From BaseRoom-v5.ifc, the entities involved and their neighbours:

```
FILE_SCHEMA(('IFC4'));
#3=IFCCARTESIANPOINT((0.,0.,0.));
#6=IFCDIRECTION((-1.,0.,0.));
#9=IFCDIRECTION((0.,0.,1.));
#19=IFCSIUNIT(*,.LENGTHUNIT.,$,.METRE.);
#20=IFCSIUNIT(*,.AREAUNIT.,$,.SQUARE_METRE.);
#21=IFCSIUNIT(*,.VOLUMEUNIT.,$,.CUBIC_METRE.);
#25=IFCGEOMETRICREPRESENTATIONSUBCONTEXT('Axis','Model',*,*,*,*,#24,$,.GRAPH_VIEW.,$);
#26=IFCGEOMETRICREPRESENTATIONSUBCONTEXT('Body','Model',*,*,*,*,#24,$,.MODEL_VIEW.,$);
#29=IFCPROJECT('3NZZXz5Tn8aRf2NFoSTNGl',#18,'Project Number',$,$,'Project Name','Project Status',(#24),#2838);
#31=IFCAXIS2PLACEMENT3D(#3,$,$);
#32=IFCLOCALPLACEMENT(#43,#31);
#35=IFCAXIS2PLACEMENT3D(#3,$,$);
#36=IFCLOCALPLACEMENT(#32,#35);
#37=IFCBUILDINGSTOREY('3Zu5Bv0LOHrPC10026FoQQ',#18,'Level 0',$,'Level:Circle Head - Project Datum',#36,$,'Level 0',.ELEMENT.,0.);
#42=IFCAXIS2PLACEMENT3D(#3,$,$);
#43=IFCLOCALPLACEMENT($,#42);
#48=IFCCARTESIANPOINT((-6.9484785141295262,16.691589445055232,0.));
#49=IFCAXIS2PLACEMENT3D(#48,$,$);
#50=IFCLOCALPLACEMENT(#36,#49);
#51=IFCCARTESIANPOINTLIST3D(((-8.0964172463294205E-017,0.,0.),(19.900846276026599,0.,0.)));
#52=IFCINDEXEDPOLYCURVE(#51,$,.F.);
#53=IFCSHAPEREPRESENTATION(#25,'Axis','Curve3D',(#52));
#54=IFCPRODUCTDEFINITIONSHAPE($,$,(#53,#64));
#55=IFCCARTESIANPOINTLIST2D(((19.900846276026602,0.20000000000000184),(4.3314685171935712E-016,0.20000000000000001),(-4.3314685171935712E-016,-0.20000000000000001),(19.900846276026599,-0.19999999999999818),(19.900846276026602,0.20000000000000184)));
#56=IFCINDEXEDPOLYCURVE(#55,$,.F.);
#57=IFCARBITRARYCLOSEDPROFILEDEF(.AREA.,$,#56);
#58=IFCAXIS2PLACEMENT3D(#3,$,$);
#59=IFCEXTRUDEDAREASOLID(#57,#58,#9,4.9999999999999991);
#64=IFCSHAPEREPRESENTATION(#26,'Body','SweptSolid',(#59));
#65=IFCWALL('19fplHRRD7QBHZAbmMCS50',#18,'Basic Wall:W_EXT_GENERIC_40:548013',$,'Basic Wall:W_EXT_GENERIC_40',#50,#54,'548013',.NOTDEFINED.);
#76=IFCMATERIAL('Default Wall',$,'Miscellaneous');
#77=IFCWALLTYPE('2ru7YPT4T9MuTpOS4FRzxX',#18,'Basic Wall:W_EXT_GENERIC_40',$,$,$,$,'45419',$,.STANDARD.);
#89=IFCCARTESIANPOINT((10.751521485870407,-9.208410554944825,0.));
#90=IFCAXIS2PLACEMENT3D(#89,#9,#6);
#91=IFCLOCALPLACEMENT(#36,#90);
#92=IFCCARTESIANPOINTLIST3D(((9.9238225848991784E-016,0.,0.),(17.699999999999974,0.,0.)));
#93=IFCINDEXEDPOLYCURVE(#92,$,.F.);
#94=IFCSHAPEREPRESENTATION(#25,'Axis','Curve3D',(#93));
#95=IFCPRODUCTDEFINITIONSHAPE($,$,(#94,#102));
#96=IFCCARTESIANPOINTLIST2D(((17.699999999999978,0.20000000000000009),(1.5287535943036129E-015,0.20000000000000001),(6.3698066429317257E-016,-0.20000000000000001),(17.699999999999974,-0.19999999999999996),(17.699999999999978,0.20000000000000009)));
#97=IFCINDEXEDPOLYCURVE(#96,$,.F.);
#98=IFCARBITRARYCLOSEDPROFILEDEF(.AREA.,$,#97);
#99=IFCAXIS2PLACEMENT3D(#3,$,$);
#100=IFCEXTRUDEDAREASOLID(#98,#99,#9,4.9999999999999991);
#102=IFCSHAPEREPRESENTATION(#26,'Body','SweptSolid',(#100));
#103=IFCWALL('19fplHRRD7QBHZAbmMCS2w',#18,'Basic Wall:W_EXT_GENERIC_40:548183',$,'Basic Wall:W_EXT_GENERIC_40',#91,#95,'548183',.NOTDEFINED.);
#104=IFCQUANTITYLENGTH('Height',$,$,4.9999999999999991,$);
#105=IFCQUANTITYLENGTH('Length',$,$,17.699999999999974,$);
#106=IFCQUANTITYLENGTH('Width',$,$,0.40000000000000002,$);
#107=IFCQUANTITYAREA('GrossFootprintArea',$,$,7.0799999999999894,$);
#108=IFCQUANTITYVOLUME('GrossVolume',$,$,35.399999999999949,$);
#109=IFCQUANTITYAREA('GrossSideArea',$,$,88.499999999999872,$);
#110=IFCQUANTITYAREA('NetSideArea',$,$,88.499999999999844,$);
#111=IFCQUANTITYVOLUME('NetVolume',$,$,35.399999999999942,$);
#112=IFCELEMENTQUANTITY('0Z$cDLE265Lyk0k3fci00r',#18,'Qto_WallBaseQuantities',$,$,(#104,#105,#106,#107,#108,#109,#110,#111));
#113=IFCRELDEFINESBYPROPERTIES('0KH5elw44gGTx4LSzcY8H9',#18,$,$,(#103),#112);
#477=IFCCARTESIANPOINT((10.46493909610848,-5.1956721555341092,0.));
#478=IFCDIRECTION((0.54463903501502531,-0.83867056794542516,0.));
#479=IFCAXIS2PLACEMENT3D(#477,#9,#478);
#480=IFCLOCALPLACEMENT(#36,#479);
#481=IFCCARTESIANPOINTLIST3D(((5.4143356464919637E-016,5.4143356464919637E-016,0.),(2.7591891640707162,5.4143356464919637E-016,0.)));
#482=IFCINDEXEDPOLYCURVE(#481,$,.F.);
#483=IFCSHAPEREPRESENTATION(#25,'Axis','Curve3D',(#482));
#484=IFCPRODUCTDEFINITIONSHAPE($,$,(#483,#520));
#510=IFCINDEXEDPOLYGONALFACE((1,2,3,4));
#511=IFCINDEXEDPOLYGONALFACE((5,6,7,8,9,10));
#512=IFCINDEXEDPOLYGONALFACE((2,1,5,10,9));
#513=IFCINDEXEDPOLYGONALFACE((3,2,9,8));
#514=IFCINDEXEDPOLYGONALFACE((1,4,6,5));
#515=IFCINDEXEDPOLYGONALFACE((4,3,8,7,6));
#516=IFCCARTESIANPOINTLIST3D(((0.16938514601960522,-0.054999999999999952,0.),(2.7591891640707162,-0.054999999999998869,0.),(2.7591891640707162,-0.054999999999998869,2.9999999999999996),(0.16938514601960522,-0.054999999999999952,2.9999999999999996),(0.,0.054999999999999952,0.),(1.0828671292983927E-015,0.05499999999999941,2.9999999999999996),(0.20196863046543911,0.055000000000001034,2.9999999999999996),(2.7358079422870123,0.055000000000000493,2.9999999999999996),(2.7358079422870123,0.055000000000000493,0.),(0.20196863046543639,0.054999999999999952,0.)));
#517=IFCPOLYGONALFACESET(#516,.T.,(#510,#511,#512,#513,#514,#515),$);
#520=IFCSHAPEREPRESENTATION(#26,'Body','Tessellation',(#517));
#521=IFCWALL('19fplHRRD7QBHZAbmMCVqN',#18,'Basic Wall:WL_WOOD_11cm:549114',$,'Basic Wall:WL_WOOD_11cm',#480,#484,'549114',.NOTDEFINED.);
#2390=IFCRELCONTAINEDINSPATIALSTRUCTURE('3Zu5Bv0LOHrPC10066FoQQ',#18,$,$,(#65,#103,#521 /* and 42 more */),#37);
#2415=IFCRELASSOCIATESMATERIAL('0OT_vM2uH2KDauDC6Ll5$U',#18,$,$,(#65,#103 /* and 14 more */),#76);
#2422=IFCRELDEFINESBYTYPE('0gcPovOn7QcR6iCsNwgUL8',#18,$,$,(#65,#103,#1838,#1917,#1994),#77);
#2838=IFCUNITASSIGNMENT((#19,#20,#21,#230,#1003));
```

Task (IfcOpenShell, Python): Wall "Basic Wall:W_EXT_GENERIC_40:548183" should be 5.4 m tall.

```python
import ifcopenshell
import ifcopenshell.api.pset
import ifcopenshell.geom
import ifcopenshell.util.element
import ifcopenshell.util.representation
import ifcopenshell.util.shape
import ifcopenshell.util.unit

model = ifcopenshell.open("BaseRoom-v5.ifc")
unit_scale = ifcopenshell.util.unit.calculate_unit_scale(model)
area_scale = ifcopenshell.util.unit.calculate_unit_scale(model, "AREAUNIT")
volume_scale = ifcopenshell.util.unit.calculate_unit_scale(model, "VOLUMEUNIT")
settings = ifcopenshell.geom.settings()


def volume(element):
    """Net volume in cubic metres, openings subtracted."""
    shape = ifcopenshell.geom.create_shape(settings, element)
    return ifcopenshell.util.shape.get_volume(shape.geometry)


wall = model.by_guid("19fplHRRD7QBHZAbmMCS2w")
before = volume(wall)

body = ifcopenshell.util.representation.get_representation(wall, "Model", "Body")
solid = body.Items[0]
old_height = solid.Depth
solid.Depth = 5.4
after = volume(wall)
thickness = 0.4  # wall thickness in metres

# Update the stored height, areas and volumes.
qto = model.by_id(ifcopenshell.util.element.get_pset(wall, "Qto_WallBaseQuantities", should_inherit=False)["id"])
ifcopenshell.api.pset.edit_qto(model, qto=qto, properties={
    "Height": solid.Depth,
    "GrossVolume": ifcopenshell.util.element.get_pset(wall, "Qto_WallBaseQuantities", "GrossVolume") * solid.Depth / old_height,
    "GrossSideArea": ifcopenshell.util.element.get_pset(wall, "Qto_WallBaseQuantities", "GrossSideArea") * solid.Depth / old_height,
    "NetSideArea": after / thickness / area_scale,
    "NetVolume": after / volume_scale,
})

print(f"height {old_height:g} -> {solid.Depth:g}, volume {before:.3f} -> {after:.3f} m3")

model.write("BaseRoom-v5_rev.ifc")
```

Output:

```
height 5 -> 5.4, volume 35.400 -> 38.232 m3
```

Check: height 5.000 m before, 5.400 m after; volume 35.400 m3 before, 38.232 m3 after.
